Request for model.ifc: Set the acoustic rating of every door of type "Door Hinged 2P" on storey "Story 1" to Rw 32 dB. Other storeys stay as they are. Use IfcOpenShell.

First a look at what the model holds.

```python
import ifcopenshell
import ifcopenshell.util.element

model = ifcopenshell.open("model.ifc")
print(model.schema)
storey = next(s for s in model.by_type("IfcBuildingStorey") if s.Name == "Story 1")
doors = [e for e in ifcopenshell.util.element.get_decomposition(storey) if e.is_a("IfcDoor")]
seen = {}
for e in doors:
    element_type = ifcopenshell.util.element.get_type(e)
    key = (element_type.Name if element_type != e and element_type else None, ifcopenshell.util.element.get_pset(e, "Pset_DoorCommon", "AcousticRating"))
    seen[key] = seen.get(key, 0) + 1
for (name, value), count in sorted(seen.items(), key=str):
    print(count, "x", name, "|", value)
```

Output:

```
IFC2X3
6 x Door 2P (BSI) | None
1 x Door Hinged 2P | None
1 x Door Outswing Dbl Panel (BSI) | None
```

```python
import ifcopenshell
import ifcopenshell.api.pset
import ifcopenshell.util.element

model = ifcopenshell.open("model.ifc")

storey = next(s for s in model.by_type("IfcBuildingStorey") if s.Name == "Story 1")
doors = [e for e in ifcopenshell.util.element.get_decomposition(storey) if e.is_a("IfcDoor")]

count = 0
for e in doors:
    element_type = ifcopenshell.util.element.get_type(e)
    if element_type in (None, e) or element_type.Name != "Door Hinged 2P":
        continue
    # add_pset returns the element's existing set when there is one.
    pset = ifcopenshell.api.pset.add_pset(model, product=e, name="Pset_DoorCommon")
    ifcopenshell.api.pset.edit_pset(model, pset=pset, properties={"AcousticRating": "Rw 32 dB"})
    count += 1

print(count, "doors updated")

model.write("model_updated.ifc")
```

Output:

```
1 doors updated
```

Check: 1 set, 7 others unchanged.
